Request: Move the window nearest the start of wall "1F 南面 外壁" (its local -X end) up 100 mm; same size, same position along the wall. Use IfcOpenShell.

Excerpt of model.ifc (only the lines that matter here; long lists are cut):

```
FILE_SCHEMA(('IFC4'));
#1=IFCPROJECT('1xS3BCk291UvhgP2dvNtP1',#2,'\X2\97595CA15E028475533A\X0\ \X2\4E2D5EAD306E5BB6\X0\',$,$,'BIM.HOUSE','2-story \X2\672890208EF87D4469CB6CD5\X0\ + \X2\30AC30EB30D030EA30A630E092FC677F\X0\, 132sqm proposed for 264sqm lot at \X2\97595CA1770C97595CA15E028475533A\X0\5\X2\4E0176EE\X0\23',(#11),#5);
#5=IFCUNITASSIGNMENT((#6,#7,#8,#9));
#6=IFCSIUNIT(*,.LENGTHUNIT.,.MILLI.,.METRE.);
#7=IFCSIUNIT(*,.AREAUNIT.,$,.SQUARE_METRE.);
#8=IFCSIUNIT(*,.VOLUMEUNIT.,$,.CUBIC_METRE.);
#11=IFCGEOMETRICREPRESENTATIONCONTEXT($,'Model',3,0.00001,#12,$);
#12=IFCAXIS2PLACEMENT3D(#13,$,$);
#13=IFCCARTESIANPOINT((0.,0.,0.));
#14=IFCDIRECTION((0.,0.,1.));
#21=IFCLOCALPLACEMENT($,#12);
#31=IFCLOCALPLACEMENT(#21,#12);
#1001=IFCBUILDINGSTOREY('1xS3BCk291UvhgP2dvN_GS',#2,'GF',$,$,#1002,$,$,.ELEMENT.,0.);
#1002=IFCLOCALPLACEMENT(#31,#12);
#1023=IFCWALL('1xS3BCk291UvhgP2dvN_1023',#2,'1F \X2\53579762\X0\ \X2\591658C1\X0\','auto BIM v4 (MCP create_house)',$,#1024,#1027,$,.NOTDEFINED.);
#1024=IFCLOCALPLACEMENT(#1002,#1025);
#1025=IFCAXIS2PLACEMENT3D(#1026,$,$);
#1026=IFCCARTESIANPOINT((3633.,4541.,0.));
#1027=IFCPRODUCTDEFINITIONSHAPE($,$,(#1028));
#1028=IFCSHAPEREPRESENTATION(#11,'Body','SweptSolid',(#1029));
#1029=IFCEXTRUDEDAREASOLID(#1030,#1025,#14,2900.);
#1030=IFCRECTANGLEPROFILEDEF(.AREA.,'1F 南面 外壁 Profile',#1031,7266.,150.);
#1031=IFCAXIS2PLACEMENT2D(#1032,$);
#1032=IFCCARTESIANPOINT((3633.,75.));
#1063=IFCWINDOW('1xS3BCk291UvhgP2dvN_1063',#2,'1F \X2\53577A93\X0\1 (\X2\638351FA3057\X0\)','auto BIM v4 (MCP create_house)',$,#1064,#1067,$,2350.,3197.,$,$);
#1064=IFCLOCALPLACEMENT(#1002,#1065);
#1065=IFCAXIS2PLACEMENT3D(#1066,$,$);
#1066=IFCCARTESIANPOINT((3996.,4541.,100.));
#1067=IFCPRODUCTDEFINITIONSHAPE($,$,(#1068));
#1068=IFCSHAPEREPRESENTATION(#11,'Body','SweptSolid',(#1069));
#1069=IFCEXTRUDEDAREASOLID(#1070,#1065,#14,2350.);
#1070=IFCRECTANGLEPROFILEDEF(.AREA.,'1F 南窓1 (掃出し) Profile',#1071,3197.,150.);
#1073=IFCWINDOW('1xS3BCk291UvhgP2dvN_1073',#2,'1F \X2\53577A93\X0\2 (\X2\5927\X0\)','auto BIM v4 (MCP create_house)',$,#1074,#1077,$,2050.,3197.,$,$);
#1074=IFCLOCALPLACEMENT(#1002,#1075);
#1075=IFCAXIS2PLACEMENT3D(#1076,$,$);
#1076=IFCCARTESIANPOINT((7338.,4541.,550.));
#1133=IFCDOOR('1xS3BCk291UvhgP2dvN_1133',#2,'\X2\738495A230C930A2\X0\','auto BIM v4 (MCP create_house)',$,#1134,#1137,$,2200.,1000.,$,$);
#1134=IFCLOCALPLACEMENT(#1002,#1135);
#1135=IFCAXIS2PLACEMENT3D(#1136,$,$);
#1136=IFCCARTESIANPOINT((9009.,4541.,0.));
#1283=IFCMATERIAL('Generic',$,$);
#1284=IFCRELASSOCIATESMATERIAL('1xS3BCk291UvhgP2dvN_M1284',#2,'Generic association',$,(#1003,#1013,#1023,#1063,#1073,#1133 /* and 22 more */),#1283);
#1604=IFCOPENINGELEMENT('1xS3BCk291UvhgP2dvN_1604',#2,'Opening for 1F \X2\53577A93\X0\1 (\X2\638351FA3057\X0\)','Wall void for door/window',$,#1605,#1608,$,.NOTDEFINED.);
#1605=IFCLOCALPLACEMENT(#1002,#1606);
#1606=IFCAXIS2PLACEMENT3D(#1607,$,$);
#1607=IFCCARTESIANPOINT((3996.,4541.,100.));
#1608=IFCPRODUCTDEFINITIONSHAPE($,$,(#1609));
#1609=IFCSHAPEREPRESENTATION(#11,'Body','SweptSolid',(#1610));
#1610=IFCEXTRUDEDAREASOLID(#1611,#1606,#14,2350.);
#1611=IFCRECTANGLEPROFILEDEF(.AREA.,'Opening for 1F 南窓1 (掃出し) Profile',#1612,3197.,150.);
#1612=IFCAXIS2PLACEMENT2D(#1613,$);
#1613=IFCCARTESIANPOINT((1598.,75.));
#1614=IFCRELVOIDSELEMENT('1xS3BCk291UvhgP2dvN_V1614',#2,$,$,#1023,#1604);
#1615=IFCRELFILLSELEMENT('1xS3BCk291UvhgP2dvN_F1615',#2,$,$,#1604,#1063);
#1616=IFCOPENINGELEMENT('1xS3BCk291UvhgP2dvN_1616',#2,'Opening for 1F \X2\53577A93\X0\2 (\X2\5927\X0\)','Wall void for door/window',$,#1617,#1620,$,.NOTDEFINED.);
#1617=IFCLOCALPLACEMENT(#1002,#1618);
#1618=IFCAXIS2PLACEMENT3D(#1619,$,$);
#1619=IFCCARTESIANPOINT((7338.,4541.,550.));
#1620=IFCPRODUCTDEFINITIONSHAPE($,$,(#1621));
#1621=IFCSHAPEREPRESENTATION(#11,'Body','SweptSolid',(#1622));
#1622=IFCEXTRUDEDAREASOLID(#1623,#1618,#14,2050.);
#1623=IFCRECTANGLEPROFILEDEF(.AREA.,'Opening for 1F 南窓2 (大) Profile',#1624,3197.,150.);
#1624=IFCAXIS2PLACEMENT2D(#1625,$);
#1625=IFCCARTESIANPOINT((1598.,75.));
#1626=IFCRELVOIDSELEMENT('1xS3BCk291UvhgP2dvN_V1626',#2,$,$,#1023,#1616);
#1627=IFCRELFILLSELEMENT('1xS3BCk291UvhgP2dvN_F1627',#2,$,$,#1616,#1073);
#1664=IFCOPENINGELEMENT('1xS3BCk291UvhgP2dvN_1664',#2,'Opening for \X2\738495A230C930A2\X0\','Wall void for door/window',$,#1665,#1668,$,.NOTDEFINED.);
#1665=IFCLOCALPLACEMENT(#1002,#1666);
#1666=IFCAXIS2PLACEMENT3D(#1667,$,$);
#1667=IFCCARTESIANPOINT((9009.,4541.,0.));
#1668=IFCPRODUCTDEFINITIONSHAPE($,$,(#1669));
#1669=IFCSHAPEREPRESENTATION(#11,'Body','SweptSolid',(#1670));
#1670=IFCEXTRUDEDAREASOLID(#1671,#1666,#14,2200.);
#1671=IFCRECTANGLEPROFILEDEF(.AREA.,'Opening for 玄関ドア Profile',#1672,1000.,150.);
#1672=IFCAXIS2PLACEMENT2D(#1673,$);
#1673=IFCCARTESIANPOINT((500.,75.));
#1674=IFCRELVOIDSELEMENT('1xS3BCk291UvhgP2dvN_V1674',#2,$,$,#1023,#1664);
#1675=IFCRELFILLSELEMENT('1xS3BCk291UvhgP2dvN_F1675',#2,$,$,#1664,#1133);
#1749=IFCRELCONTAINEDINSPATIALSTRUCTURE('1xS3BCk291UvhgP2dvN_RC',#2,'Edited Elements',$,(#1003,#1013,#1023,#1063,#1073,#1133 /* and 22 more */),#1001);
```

```python
import numpy as np
import ifcopenshell
import ifcopenshell.api.geometry
import ifcopenshell.util.placement
import ifcopenshell.util.unit

model = ifcopenshell.open("model.ifc")
unit_scale = ifcopenshell.util.unit.calculate_unit_scale(model)

window = model.by_id(1063)
opening = window.FillsVoids[0].RelatingOpeningElement
dz = 100.0

shift = np.array([0.0, 0.0, dz])
# The window is not placed relative to its opening, so move both.
for product in (opening, window):
    matrix = ifcopenshell.util.placement.get_local_placement(product.ObjectPlacement)
    matrix[:3, 3] += shift
    ifcopenshell.api.geometry.edit_object_placement(model, product=product, matrix=matrix, is_si=False)

print(f"moved by {dz * unit_scale:+.3f} m")

model.write("model_updated.ifc")
```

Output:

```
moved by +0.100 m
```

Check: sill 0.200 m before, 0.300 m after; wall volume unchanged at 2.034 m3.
